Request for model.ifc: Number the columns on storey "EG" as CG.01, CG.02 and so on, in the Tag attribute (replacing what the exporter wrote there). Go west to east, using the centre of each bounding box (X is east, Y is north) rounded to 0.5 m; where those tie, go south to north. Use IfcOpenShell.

First a look at what the model holds.

```python
import ifcopenshell
import ifcopenshell.util.element
import ifcopenshell.util.placement

model = ifcopenshell.open("model.ifc")
print(model.schema)
storey = next(s for s in model.by_type("IfcBuildingStorey") if s.Name == "EG")
columns = [e for e in ifcopenshell.util.element.get_decomposition(storey) if e.is_a("IfcColumn")]
for e in sorted(columns, key=lambda e: e.id()):
    origin = ifcopenshell.util.placement.get_local_placement(e.ObjectPlacement)[:3, 3]
    print(e.id(), e.Tag, e.Name, origin.round(2) + 0.0, sep=" | ")
```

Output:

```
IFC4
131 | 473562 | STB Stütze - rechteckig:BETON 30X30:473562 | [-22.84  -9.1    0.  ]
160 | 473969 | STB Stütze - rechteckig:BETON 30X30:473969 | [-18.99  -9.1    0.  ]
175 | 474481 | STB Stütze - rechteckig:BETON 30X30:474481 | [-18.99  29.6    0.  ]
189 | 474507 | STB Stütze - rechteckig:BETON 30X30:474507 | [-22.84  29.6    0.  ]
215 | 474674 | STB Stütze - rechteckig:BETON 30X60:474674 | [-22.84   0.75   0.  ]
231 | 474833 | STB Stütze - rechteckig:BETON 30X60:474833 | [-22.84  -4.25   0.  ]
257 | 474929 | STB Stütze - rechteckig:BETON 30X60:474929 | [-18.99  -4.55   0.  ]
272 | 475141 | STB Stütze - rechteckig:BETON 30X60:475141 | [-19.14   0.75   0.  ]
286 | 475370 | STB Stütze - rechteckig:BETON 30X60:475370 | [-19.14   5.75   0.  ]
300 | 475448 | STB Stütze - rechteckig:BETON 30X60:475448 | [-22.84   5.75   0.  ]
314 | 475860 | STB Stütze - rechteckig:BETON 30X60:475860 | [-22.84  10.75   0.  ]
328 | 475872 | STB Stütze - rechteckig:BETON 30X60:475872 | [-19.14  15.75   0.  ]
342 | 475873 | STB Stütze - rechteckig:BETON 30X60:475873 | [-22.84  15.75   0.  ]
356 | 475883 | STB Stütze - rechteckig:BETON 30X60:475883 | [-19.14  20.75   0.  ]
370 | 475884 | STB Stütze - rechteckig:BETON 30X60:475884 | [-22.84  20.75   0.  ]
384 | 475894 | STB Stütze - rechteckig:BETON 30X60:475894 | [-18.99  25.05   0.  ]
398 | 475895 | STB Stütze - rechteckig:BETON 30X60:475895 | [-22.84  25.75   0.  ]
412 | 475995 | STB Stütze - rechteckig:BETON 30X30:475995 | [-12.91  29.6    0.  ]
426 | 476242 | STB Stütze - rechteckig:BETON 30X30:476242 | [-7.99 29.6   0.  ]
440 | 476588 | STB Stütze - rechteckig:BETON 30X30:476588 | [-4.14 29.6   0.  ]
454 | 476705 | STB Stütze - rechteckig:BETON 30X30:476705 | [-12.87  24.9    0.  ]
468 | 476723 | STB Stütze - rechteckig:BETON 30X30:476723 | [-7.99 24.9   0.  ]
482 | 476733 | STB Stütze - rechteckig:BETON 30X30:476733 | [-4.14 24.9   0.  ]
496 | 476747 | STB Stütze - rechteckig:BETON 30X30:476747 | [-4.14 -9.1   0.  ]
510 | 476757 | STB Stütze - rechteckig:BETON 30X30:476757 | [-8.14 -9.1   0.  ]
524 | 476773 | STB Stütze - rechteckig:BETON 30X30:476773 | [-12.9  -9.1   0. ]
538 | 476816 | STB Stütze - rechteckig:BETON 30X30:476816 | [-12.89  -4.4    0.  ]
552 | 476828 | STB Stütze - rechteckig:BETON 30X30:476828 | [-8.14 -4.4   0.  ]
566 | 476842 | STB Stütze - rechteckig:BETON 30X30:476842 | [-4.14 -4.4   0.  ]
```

```python
import ifcopenshell
import ifcopenshell.geom
import ifcopenshell.util.element
import ifcopenshell.util.shape

model = ifcopenshell.open("model.ifc")
settings = ifcopenshell.geom.settings()
settings.set("use-world-coords", True)


def centre(element):
    shape = ifcopenshell.geom.create_shape(settings, element)
    return ifcopenshell.util.shape.get_bbox_centroid(shape.geometry)


storey = next(s for s in model.by_type("IfcBuildingStorey") if s.Name == "EG")
columns = [e for e in ifcopenshell.util.element.get_decomposition(storey) if e.is_a("IfcColumn")]

# Insertion points can sit at a corner or the storey origin, so sort by the geometry (in metres).
centres = {e: centre(e) for e in columns}
columns.sort(key=lambda e: (round(centres[e][0] / 0.5), centres[e][1]))

for i, e in enumerate(columns, start=1):
    number = f"CG.{i:02d}"
    e.Tag = number
    print(e.id(), number)

model.write("model_v2.ifc")
```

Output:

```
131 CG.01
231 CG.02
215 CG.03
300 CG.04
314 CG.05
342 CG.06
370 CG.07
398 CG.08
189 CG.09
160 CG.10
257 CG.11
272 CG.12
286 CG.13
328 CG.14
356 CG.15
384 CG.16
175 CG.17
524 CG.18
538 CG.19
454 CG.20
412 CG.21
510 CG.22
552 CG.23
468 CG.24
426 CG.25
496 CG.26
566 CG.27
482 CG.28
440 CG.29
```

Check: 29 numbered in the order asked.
